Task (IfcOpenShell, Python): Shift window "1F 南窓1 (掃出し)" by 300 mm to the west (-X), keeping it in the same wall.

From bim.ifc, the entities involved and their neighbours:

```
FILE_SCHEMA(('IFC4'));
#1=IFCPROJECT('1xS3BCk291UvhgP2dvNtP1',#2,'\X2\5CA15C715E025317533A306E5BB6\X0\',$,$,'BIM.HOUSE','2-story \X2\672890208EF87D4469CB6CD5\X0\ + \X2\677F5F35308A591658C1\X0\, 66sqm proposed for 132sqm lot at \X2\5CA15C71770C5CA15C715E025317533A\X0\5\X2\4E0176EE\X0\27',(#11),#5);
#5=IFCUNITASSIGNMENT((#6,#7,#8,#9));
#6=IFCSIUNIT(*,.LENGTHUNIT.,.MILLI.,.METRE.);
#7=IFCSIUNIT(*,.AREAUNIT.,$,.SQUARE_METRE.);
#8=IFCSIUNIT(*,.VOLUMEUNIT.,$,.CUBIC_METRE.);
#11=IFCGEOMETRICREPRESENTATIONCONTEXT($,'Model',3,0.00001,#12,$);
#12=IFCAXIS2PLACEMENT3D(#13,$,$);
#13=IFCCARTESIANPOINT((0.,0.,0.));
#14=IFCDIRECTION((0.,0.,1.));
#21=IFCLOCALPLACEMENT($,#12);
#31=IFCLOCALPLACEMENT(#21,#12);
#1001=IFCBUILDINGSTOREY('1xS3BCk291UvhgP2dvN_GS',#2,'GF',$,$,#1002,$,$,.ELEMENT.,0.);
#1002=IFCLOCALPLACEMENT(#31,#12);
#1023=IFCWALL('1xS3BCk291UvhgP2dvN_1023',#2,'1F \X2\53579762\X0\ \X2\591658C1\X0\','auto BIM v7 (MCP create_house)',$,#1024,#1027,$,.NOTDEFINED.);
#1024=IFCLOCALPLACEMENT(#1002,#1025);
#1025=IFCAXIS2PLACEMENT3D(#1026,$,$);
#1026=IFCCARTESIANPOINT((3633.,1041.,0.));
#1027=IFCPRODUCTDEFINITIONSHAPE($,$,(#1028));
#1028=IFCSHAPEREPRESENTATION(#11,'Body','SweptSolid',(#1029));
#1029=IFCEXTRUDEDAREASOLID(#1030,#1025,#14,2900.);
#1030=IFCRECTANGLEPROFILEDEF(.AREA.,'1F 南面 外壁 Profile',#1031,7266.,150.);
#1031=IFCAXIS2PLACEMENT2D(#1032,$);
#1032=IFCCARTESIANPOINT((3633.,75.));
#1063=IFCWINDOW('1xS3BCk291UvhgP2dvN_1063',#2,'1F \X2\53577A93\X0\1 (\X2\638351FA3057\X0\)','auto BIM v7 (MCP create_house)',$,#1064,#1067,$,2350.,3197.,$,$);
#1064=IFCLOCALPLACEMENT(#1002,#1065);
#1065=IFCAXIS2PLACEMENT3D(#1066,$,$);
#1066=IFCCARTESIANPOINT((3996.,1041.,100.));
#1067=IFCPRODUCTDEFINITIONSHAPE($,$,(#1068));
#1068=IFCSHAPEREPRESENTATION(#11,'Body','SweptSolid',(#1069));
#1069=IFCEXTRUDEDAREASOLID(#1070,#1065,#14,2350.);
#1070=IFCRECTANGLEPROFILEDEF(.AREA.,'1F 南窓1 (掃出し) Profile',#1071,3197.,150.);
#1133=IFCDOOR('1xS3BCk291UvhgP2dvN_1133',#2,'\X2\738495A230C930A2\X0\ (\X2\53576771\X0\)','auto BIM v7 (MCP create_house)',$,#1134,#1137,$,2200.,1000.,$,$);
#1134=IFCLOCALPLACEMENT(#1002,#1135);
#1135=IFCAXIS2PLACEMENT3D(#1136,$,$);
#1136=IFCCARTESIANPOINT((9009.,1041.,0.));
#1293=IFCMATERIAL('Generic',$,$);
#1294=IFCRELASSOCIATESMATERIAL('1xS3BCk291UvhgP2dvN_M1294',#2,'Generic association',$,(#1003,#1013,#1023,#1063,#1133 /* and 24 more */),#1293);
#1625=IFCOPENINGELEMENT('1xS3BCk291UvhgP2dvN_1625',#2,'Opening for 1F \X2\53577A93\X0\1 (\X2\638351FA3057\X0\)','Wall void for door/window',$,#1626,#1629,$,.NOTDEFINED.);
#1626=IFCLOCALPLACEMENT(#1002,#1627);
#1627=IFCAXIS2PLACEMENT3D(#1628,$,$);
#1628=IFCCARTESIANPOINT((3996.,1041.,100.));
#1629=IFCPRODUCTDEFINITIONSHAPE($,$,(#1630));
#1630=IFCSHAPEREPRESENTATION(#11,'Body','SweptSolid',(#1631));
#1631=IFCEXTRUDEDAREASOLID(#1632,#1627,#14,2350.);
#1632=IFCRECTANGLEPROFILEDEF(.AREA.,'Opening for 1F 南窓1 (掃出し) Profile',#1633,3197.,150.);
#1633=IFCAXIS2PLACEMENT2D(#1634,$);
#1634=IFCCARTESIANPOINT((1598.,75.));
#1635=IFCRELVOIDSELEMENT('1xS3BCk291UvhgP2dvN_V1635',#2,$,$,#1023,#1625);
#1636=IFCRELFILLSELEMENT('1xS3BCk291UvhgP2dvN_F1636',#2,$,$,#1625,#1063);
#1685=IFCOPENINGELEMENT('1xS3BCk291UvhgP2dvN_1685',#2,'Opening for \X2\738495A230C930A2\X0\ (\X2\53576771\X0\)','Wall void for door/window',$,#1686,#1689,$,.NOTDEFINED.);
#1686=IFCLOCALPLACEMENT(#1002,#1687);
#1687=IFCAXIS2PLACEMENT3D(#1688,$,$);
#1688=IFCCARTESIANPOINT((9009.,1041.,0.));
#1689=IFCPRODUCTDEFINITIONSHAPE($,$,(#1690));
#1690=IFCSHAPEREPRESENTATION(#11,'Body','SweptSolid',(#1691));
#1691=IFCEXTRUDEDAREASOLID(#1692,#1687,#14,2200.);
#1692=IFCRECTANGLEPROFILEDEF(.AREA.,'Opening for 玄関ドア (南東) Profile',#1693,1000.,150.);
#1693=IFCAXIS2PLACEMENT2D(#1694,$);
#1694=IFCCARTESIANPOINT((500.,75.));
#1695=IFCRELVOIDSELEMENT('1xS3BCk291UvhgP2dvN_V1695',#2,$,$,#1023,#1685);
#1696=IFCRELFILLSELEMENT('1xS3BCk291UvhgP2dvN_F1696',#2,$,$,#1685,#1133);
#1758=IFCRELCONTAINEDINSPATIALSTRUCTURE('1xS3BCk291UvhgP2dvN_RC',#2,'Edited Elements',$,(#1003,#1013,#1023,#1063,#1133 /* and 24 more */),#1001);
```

```python
import ifcopenshell
import ifcopenshell.api.geometry
import ifcopenshell.util.placement
import ifcopenshell.util.unit

model = ifcopenshell.open("bim.ifc")
unit_scale = ifcopenshell.util.unit.calculate_unit_scale(model)

window = model.by_guid("1xS3BCk291UvhgP2dvN_1063")
opening = window.FillsVoids[0].RelatingOpeningElement
wall = opening.VoidsElements[0].RelatingBuildingElement

wall_matrix = ifcopenshell.util.placement.get_local_placement(wall.ObjectPlacement)
shift = wall_matrix[:3, 0] * -0.3 / unit_scale
before = ifcopenshell.util.placement.get_local_placement(window.ObjectPlacement)[:3, 3].copy()

# The window is not placed relative to its opening, so move both.
for product in (opening, window):
    matrix = ifcopenshell.util.placement.get_local_placement(product.ObjectPlacement)
    matrix[:3, 3] += shift
    ifcopenshell.api.geometry.edit_object_placement(model, product=product, matrix=matrix, is_si=False)

after = ifcopenshell.util.placement.get_local_placement(window.ObjectPlacement)[:3, 3]
print("window moved by", (after - before).round(3) + 0.0)

model.write("bim_v2.ifc")
```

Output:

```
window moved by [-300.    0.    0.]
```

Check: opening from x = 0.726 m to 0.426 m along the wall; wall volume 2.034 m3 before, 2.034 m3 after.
